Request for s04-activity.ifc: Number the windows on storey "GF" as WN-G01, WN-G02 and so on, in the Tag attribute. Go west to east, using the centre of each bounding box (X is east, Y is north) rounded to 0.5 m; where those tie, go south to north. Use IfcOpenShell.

First a look at what the model holds.

```python
import ifcopenshell
import ifcopenshell.util.element
import ifcopenshell.util.placement

model = ifcopenshell.open("s04-activity.ifc")
print(model.schema)
storey = next(s for s in model.by_type("IfcBuildingStorey") if s.Name == "GF")
windows = [e for e in ifcopenshell.util.element.get_decomposition(storey) if e.is_a("IfcWindow")]
for e in sorted(windows, key=lambda e: e.id()):
    origin = ifcopenshell.util.placement.get_local_placement(e.ObjectPlacement)[:3, 3]
    print(e.id(), e.Tag, e.Name, origin.round(2) + 0.0, sep=" | ")
```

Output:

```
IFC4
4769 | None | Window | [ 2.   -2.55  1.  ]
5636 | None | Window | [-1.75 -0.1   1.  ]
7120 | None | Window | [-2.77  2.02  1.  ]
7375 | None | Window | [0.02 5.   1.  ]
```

```python
import ifcopenshell
import ifcopenshell.geom
import ifcopenshell.util.element
import ifcopenshell.util.shape

model = ifcopenshell.open("s04-activity.ifc")
settings = ifcopenshell.geom.settings()
settings.set("use-world-coords", True)


def centre(element):
    shape = ifcopenshell.geom.create_shape(settings, element)
    return ifcopenshell.util.shape.get_bbox_centroid(shape.geometry)


storey = next(s for s in model.by_type("IfcBuildingStorey") if s.Name == "GF")
windows = [e for e in ifcopenshell.util.element.get_decomposition(storey) if e.is_a("IfcWindow")]

# Insertion points can sit at a corner or the storey origin, so sort by the geometry (in metres).
centres = {e: centre(e) for e in windows}
windows.sort(key=lambda e: (round(centres[e][0] / 0.5), centres[e][1]))

for i, e in enumerate(windows, start=1):
    number = f"WN-G{i:02d}"
    e.Tag = number
    print(e.id(), number)

model.write("s04-activity_edited.ifc")
```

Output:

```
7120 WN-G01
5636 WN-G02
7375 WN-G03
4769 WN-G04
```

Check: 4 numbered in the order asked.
